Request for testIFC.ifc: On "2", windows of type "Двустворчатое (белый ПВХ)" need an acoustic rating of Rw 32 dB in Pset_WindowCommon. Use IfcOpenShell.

First a look at what the model holds.

```python
import ifcopenshell
import ifcopenshell.util.element

model = ifcopenshell.open("testIFC.ifc")
print(model.schema)
storey = next(s for s in model.by_type("IfcBuildingStorey") if s.Name == "2")
windows = [e for e in ifcopenshell.util.element.get_decomposition(storey) if e.is_a("IfcWindow")]
seen = {}
for e in windows:
    element_type = ifcopenshell.util.element.get_type(e)
    key = (element_type.Name if element_type != e and element_type else None, ifcopenshell.util.element.get_pset(e, "Pset_WindowCommon", "AcousticRating"))
    seen[key] = seen.get(key, 0) + 1
for (name, value), count in sorted(seen.items(), key=str):
    print(count, "x", name, "|", value)
```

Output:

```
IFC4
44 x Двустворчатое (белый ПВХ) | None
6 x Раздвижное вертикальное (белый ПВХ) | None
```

```python
import ifcopenshell
import ifcopenshell.api.pset
import ifcopenshell.util.element

model = ifcopenshell.open("testIFC.ifc")

storey = next(s for s in model.by_type("IfcBuildingStorey") if s.Name == "2")
windows = [e for e in ifcopenshell.util.element.get_decomposition(storey) if e.is_a("IfcWindow")]

count = 0
for e in windows:
    element_type = ifcopenshell.util.element.get_type(e)
    if element_type in (None, e) or element_type.Name != "Двустворчатое (белый ПВХ)":
        continue
    # add_pset returns the element's existing set when there is one.
    pset = ifcopenshell.api.pset.add_pset(model, product=e, name="Pset_WindowCommon")
    ifcopenshell.api.pset.edit_pset(model, pset=pset, properties={"AcousticRating": "Rw 32 dB"})
    count += 1

print(count, "windows updated")

model.write("testIFC_v2.ifc")
```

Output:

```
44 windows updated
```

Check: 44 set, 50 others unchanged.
